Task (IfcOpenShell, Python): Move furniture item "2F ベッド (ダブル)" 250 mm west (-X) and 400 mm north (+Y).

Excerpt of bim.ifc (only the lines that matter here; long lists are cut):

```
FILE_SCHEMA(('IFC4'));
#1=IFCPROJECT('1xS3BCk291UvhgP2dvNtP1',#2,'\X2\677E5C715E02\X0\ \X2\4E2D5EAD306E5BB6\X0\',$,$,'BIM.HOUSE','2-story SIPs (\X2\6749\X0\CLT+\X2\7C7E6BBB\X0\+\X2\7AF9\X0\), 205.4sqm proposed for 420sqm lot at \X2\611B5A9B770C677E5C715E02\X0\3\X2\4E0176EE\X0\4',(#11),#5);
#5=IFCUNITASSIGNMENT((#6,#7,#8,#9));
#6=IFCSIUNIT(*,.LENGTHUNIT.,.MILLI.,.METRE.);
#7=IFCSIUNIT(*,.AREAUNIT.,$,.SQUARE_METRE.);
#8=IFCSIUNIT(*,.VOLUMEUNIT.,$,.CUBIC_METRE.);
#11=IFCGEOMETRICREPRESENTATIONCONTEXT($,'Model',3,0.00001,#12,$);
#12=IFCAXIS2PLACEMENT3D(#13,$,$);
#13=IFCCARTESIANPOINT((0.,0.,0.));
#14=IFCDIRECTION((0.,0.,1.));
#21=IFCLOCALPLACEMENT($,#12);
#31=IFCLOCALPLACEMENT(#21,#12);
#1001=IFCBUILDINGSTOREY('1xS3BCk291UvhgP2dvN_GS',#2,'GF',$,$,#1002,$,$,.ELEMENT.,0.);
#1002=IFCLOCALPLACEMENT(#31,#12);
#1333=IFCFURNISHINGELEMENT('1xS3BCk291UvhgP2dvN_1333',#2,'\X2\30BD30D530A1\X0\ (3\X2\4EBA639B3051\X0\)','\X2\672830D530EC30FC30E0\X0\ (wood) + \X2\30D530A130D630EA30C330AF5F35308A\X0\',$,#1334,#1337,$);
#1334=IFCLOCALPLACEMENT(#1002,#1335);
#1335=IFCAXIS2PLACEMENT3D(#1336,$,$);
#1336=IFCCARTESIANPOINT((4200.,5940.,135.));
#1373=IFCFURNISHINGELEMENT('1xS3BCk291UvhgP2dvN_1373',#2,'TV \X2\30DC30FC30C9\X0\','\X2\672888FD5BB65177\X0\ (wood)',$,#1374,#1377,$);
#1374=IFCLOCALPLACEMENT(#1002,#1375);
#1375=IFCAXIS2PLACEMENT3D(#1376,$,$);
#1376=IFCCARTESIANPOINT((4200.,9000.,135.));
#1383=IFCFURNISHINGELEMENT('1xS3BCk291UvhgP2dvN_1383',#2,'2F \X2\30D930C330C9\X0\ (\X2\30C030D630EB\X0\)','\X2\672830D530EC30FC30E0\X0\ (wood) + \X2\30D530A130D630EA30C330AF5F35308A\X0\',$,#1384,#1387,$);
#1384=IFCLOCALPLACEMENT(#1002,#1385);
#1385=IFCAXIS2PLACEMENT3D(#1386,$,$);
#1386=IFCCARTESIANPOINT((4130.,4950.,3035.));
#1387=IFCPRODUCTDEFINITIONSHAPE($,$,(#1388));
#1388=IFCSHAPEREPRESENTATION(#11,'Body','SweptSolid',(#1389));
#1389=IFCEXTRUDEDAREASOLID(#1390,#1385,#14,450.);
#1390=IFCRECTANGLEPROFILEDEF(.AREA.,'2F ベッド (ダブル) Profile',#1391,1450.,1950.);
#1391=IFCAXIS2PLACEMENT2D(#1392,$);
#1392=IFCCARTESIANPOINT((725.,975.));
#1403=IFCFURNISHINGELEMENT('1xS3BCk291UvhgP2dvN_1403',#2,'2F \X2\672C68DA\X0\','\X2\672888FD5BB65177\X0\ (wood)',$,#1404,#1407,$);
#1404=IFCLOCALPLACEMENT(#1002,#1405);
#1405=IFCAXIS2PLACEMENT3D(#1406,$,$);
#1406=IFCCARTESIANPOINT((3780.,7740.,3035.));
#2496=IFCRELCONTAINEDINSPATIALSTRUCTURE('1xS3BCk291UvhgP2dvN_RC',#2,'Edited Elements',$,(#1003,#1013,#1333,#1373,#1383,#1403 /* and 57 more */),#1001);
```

```python
import ifcopenshell
import ifcopenshell.api.geometry
import ifcopenshell.util.placement
import ifcopenshell.util.unit

model = ifcopenshell.open("bim.ifc")
unit_scale = ifcopenshell.util.unit.calculate_unit_scale(model)

item = model.by_guid("1xS3BCk291UvhgP2dvN_1383")
matrix = ifcopenshell.util.placement.get_local_placement(item.ObjectPlacement)
matrix[0, 3] -= 0.25 / unit_scale
matrix[1, 3] += 0.4 / unit_scale
ifcopenshell.api.geometry.edit_object_placement(model, product=item, matrix=matrix, is_si=False)

print(ifcopenshell.util.placement.get_local_placement(item.ObjectPlacement).round(3) + 0.0)

model.write("bim_edited.ifc")
```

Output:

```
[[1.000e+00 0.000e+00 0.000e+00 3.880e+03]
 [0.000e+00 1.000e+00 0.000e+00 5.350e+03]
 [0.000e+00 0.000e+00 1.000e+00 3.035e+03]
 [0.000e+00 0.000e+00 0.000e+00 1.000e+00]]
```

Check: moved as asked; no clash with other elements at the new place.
